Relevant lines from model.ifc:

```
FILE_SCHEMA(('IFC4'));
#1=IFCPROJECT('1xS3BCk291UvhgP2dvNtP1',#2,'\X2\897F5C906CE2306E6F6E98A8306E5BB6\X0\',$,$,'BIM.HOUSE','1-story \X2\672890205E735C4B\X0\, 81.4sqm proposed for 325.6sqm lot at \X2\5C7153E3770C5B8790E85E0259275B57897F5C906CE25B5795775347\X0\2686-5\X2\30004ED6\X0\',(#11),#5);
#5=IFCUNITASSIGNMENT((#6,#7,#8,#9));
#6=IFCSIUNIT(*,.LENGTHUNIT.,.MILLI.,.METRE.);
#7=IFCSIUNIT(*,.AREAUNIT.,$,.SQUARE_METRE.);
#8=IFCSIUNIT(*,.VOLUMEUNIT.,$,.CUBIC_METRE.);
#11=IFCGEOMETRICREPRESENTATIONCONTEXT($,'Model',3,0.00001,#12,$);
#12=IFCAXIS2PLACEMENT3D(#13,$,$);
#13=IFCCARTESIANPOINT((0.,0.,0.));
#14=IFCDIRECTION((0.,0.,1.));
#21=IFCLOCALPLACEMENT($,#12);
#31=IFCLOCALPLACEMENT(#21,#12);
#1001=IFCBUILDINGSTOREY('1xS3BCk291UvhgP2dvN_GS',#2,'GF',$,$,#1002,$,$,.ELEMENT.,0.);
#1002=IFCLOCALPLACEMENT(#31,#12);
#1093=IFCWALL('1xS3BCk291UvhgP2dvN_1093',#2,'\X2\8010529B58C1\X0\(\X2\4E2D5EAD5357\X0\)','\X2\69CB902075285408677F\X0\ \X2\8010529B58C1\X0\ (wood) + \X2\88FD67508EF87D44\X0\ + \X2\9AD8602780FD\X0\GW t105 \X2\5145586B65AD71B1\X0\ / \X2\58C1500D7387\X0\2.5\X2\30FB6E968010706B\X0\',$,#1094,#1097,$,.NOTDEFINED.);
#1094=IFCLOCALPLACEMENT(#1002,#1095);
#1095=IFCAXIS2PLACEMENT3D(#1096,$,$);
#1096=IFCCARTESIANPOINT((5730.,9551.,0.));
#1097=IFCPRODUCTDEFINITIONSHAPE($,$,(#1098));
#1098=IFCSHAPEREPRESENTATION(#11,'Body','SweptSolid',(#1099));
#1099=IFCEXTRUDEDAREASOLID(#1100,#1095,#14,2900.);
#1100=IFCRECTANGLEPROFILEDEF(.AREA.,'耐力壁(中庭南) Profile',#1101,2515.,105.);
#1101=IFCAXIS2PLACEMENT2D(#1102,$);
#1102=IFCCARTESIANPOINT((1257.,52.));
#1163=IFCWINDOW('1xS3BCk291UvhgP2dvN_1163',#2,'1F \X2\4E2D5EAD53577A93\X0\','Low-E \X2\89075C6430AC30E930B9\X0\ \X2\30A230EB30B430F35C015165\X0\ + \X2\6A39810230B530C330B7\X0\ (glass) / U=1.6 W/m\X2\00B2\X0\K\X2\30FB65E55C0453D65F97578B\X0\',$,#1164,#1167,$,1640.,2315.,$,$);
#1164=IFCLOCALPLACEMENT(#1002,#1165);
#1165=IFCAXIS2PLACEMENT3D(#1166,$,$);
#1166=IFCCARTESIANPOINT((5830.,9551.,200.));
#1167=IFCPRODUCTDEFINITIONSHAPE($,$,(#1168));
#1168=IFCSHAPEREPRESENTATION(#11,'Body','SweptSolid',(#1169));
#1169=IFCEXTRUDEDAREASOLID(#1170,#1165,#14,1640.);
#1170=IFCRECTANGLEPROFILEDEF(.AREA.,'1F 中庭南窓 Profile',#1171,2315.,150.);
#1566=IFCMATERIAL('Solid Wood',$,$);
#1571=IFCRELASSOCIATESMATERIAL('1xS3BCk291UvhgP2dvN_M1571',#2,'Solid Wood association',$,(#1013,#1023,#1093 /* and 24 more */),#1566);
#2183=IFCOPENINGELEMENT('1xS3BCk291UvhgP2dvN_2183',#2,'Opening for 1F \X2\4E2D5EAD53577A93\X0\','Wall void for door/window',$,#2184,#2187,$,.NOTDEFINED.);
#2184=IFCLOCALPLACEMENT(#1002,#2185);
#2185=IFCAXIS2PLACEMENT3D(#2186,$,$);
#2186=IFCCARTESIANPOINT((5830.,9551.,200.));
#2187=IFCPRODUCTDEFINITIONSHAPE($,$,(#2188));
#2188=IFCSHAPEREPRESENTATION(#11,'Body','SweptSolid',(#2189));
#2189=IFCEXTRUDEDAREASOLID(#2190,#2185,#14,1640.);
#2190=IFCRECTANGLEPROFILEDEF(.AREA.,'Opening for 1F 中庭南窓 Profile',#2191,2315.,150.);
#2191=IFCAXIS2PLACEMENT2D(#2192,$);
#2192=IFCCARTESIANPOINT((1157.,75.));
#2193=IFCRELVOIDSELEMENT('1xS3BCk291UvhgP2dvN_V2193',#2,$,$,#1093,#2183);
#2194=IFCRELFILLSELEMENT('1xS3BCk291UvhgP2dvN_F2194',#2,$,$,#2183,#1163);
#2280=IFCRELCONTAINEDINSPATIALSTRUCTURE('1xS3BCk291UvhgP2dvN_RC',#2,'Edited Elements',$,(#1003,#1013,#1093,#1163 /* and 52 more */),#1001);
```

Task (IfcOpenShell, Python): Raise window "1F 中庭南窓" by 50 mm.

```python
import numpy as np
import ifcopenshell
import ifcopenshell.api.geometry
import ifcopenshell.util.placement
import ifcopenshell.util.unit

model = ifcopenshell.open("model.ifc")
unit_scale = ifcopenshell.util.unit.calculate_unit_scale(model)

window = model.by_guid("1xS3BCk291UvhgP2dvN_1163")
opening = window.FillsVoids[0].RelatingOpeningElement
dz = 0.05 / unit_scale

shift = np.array([0.0, 0.0, dz])
# The window is not placed relative to its opening, so move both.
for product in (opening, window):
    matrix = ifcopenshell.util.placement.get_local_placement(product.ObjectPlacement)
    matrix[:3, 3] += shift
    ifcopenshell.api.geometry.edit_object_placement(model, product=product, matrix=matrix, is_si=False)

print(f"moved by {dz * unit_scale:+.3f} m")

model.write("model_v2.ifc")
```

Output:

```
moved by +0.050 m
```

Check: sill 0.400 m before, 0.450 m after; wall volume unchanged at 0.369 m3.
